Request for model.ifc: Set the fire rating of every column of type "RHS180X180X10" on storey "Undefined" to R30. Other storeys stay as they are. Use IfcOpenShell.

First a look at what the model holds.

```python
import ifcopenshell
import ifcopenshell.util.element

model = ifcopenshell.open("model.ifc")
print(model.schema)
storey = next(s for s in model.by_type("IfcBuildingStorey") if s.Name == "Undefined")
columns = [e for e in ifcopenshell.util.element.get_decomposition(storey) if e.is_a("IfcColumn")]
seen = {}
for e in columns:
    element_type = ifcopenshell.util.element.get_type(e)
    key = (element_type.Name if element_type != e and element_type else None, ifcopenshell.util.element.get_pset(e, "Pset_ColumnCommon", "FireRating"))
    seen[key] = seen.get(key, 0) + 1
for (name, value), count in sorted(seen.items(), key=str):
    print(count, "x", name, "|", value)
```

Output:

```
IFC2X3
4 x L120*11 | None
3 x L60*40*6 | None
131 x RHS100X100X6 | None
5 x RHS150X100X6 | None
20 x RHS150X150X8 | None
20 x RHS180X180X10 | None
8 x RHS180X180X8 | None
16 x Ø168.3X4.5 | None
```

```python
import ifcopenshell
import ifcopenshell.api.pset
import ifcopenshell.util.element

model = ifcopenshell.open("model.ifc")

storey = next(s for s in model.by_type("IfcBuildingStorey") if s.Name == "Undefined")
columns = [e for e in ifcopenshell.util.element.get_decomposition(storey) if e.is_a("IfcColumn")]

count = 0
for e in columns:
    element_type = ifcopenshell.util.element.get_type(e)
    if element_type in (None, e) or element_type.Name != "RHS180X180X10":
        continue
    found = ifcopenshell.util.element.get_pset(e, "Pset_ColumnCommon", should_inherit=False)
    if found:
        pset = model.by_id(found["id"])
        if len(ifcopenshell.util.element.get_elements_by_pset(pset)) > 1:
            pset = ifcopenshell.api.pset.unshare_pset(model, products=[e], pset=pset)[0]
    else:
        pset = ifcopenshell.api.pset.add_pset(model, product=e, name="Pset_ColumnCommon")
    ifcopenshell.api.pset.edit_pset(model, pset=pset, properties={"FireRating": "R30"})
    count += 1

print(count, "columns updated")

model.write("model_edited.ifc")
```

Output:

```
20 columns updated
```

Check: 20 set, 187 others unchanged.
